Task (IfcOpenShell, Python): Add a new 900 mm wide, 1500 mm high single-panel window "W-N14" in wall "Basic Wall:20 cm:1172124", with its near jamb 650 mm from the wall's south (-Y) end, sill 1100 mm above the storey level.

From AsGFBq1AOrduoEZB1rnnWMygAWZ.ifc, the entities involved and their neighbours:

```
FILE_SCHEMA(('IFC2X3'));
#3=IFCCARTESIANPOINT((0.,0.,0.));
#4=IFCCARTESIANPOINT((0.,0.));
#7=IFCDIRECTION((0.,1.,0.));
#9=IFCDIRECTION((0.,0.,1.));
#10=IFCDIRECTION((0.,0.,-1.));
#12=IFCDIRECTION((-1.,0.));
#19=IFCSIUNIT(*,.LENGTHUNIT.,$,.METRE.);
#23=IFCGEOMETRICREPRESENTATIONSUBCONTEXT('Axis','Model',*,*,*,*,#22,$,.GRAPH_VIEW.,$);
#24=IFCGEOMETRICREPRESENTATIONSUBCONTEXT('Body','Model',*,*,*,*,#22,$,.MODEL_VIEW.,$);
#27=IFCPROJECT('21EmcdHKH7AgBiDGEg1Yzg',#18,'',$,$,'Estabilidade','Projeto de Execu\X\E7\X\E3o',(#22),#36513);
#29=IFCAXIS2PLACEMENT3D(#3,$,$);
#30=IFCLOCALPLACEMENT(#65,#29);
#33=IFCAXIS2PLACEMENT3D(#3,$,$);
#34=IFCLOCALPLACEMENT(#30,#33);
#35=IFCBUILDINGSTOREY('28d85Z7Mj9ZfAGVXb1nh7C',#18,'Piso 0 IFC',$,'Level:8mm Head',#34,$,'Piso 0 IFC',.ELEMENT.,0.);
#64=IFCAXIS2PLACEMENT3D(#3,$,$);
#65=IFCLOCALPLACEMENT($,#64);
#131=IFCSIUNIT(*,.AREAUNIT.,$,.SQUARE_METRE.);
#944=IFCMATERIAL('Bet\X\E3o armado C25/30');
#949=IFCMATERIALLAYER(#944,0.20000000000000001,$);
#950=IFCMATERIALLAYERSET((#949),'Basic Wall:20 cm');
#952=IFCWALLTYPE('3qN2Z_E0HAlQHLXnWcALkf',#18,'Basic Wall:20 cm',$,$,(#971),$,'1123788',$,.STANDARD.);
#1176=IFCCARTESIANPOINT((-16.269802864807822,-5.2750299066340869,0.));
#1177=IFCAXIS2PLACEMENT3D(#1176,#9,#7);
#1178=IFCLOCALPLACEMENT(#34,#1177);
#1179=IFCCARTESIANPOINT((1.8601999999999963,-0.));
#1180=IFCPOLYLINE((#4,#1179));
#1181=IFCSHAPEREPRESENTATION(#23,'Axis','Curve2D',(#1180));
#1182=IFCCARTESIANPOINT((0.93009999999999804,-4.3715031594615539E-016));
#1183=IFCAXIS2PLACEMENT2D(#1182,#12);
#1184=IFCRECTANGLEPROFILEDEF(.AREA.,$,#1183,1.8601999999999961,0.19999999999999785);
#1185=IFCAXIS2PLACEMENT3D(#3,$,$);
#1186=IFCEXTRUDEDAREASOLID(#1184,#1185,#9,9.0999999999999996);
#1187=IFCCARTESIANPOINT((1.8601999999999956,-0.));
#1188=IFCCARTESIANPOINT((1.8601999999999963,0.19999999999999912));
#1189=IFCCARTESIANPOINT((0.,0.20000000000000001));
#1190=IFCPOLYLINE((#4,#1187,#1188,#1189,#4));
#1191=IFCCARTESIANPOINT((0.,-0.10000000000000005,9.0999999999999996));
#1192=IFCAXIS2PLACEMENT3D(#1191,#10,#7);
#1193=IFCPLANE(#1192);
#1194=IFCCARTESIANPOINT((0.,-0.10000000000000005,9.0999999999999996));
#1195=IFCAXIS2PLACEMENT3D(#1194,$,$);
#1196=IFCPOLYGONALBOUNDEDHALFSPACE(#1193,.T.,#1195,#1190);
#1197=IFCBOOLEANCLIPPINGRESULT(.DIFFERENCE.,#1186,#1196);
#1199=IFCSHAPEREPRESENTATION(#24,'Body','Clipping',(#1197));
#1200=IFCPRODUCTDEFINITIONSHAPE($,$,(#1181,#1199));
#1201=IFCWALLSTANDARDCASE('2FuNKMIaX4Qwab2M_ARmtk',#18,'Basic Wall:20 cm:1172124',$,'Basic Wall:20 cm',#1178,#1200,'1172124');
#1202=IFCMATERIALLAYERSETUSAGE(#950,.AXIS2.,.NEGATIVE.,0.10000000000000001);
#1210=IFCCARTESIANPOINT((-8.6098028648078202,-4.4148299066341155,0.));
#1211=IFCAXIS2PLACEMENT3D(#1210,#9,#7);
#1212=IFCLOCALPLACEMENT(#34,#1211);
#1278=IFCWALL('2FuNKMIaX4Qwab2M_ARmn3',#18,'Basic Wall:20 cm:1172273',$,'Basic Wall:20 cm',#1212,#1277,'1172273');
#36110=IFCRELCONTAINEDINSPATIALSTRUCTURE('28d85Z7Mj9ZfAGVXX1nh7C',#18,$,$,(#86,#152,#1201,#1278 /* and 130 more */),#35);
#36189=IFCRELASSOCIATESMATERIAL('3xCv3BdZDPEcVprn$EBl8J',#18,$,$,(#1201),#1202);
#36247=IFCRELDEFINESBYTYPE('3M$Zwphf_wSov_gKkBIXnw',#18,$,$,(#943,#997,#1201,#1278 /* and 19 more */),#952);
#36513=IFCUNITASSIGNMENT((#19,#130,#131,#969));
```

```python
import numpy as np
import ifcopenshell
import ifcopenshell.api.feature
import ifcopenshell.api.geometry
import ifcopenshell.api.root
import ifcopenshell.api.spatial
import ifcopenshell.api.type
import ifcopenshell.geom
import ifcopenshell.util.element
import ifcopenshell.util.placement
import ifcopenshell.util.representation
import ifcopenshell.util.shape
import ifcopenshell.util.unit

model = ifcopenshell.open("AsGFBq1AOrduoEZB1rnnWMygAWZ.ifc")
unit_scale = ifcopenshell.util.unit.calculate_unit_scale(model)
settings = ifcopenshell.geom.settings()


def volume(element):
    """Net volume in cubic metres, openings subtracted."""
    shape = ifcopenshell.geom.create_shape(settings, element)
    return ifcopenshell.util.shape.get_volume(shape.geometry)


wall = model.by_guid("2FuNKMIaX4Qwab2M_ARmtk")
storey = ifcopenshell.util.element.get_container(wall, ifc_class="IfcBuildingStorey")
context = ifcopenshell.util.representation.get_context(model, "Model", "Body", "MODEL_VIEW")
before = volume(wall)

width, height, from_end, sill = 0.9, 1.5, 0.65, 1.1  # metres

# The wall runs along its own X axis, and the end named is its -X end.
wall_shape = ifcopenshell.geom.create_shape(settings, wall)
x, y, z = ifcopenshell.util.shape.get_vertices(wall_shape.geometry).T
start = x.min() + from_end
face, thickness = float(y.min()), float(y.max() - y.min())
wall_matrix = ifcopenshell.util.placement.get_local_placement(wall.ObjectPlacement)
level = ifcopenshell.util.placement.get_local_placement(storey.ObjectPlacement)[2, 3]


def in_wall(x, y):
    """Placement at x, y metres in the wall's axes, at sill height."""
    matrix = wall_matrix.copy()
    matrix[:, 3] = wall_matrix @ np.array([x / unit_scale, y / unit_scale, 0.0, 1.0])
    matrix[2, 3] = level + sill / unit_scale
    return matrix


# Opening: a box that overshoots both wall faces by 50 mm.
opening = ifcopenshell.api.root.create_entity(model, ifc_class="IfcOpeningElement")
box = ifcopenshell.api.geometry.add_wall_representation(
    model, context=context, length=width, height=height, thickness=thickness + 0.1
)
ifcopenshell.api.geometry.assign_representation(model, product=opening, representation=box)
ifcopenshell.api.geometry.edit_object_placement(model, product=opening, matrix=in_wall(start, face - 0.05), is_si=False)
ifcopenshell.api.feature.add_feature(model, feature=opening, element=wall)

window = ifcopenshell.api.root.create_entity(model, ifc_class="IfcWindow", name="W-N14")
window.OverallWidth, window.OverallHeight = width / unit_scale, height / unit_scale
body = ifcopenshell.api.geometry.add_window_representation(
    model,
    context=context,
    overall_width=window.OverallWidth,
    overall_height=window.OverallHeight,
    partition_type="SINGLE_PANEL",
)
ifcopenshell.api.geometry.assign_representation(model, product=window, representation=body)
ifcopenshell.api.spatial.assign_container(model, products=[window], relating_structure=storey)
fills = ifcopenshell.api.feature.add_filling(model, opening=opening, element=window)
fills.OwnerHistory = window.OwnerHistory  # required in IFC2X3

# IFC2X3 keeps the operation on the window style.
style = ifcopenshell.api.root.create_entity(model, ifc_class="IfcWindowStyle", name="W-N14")
style.OperationType, style.ConstructionType = "SINGLE_PANEL", "NOTDEFINED"
style.ParameterTakesPrecedence = style.Sizeable = False
ifcopenshell.api.type.assign_type(model, related_objects=[window], relating_type=style)

# Centre the window in the wall's thickness.
ifcopenshell.api.geometry.edit_object_placement(model, product=window, matrix=in_wall(start, face), is_si=False)
window_shape = ifcopenshell.geom.create_shape(settings, window)
depth = ifcopenshell.util.shape.get_vertices(window_shape.geometry)[:, 1]
offset = face + thickness / 2 - (depth.min() + depth.max()) / 2
ifcopenshell.api.geometry.edit_object_placement(model, product=window, matrix=in_wall(start, offset), is_si=False)

after = volume(wall)

print(f"wall volume {before:.3f} -> {after:.3f} m3")

model.write("AsGFBq1AOrduoEZB1rnnWMygAWZ_rev.ifc")
```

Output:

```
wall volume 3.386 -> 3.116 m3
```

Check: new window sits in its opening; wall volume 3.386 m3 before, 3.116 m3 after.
